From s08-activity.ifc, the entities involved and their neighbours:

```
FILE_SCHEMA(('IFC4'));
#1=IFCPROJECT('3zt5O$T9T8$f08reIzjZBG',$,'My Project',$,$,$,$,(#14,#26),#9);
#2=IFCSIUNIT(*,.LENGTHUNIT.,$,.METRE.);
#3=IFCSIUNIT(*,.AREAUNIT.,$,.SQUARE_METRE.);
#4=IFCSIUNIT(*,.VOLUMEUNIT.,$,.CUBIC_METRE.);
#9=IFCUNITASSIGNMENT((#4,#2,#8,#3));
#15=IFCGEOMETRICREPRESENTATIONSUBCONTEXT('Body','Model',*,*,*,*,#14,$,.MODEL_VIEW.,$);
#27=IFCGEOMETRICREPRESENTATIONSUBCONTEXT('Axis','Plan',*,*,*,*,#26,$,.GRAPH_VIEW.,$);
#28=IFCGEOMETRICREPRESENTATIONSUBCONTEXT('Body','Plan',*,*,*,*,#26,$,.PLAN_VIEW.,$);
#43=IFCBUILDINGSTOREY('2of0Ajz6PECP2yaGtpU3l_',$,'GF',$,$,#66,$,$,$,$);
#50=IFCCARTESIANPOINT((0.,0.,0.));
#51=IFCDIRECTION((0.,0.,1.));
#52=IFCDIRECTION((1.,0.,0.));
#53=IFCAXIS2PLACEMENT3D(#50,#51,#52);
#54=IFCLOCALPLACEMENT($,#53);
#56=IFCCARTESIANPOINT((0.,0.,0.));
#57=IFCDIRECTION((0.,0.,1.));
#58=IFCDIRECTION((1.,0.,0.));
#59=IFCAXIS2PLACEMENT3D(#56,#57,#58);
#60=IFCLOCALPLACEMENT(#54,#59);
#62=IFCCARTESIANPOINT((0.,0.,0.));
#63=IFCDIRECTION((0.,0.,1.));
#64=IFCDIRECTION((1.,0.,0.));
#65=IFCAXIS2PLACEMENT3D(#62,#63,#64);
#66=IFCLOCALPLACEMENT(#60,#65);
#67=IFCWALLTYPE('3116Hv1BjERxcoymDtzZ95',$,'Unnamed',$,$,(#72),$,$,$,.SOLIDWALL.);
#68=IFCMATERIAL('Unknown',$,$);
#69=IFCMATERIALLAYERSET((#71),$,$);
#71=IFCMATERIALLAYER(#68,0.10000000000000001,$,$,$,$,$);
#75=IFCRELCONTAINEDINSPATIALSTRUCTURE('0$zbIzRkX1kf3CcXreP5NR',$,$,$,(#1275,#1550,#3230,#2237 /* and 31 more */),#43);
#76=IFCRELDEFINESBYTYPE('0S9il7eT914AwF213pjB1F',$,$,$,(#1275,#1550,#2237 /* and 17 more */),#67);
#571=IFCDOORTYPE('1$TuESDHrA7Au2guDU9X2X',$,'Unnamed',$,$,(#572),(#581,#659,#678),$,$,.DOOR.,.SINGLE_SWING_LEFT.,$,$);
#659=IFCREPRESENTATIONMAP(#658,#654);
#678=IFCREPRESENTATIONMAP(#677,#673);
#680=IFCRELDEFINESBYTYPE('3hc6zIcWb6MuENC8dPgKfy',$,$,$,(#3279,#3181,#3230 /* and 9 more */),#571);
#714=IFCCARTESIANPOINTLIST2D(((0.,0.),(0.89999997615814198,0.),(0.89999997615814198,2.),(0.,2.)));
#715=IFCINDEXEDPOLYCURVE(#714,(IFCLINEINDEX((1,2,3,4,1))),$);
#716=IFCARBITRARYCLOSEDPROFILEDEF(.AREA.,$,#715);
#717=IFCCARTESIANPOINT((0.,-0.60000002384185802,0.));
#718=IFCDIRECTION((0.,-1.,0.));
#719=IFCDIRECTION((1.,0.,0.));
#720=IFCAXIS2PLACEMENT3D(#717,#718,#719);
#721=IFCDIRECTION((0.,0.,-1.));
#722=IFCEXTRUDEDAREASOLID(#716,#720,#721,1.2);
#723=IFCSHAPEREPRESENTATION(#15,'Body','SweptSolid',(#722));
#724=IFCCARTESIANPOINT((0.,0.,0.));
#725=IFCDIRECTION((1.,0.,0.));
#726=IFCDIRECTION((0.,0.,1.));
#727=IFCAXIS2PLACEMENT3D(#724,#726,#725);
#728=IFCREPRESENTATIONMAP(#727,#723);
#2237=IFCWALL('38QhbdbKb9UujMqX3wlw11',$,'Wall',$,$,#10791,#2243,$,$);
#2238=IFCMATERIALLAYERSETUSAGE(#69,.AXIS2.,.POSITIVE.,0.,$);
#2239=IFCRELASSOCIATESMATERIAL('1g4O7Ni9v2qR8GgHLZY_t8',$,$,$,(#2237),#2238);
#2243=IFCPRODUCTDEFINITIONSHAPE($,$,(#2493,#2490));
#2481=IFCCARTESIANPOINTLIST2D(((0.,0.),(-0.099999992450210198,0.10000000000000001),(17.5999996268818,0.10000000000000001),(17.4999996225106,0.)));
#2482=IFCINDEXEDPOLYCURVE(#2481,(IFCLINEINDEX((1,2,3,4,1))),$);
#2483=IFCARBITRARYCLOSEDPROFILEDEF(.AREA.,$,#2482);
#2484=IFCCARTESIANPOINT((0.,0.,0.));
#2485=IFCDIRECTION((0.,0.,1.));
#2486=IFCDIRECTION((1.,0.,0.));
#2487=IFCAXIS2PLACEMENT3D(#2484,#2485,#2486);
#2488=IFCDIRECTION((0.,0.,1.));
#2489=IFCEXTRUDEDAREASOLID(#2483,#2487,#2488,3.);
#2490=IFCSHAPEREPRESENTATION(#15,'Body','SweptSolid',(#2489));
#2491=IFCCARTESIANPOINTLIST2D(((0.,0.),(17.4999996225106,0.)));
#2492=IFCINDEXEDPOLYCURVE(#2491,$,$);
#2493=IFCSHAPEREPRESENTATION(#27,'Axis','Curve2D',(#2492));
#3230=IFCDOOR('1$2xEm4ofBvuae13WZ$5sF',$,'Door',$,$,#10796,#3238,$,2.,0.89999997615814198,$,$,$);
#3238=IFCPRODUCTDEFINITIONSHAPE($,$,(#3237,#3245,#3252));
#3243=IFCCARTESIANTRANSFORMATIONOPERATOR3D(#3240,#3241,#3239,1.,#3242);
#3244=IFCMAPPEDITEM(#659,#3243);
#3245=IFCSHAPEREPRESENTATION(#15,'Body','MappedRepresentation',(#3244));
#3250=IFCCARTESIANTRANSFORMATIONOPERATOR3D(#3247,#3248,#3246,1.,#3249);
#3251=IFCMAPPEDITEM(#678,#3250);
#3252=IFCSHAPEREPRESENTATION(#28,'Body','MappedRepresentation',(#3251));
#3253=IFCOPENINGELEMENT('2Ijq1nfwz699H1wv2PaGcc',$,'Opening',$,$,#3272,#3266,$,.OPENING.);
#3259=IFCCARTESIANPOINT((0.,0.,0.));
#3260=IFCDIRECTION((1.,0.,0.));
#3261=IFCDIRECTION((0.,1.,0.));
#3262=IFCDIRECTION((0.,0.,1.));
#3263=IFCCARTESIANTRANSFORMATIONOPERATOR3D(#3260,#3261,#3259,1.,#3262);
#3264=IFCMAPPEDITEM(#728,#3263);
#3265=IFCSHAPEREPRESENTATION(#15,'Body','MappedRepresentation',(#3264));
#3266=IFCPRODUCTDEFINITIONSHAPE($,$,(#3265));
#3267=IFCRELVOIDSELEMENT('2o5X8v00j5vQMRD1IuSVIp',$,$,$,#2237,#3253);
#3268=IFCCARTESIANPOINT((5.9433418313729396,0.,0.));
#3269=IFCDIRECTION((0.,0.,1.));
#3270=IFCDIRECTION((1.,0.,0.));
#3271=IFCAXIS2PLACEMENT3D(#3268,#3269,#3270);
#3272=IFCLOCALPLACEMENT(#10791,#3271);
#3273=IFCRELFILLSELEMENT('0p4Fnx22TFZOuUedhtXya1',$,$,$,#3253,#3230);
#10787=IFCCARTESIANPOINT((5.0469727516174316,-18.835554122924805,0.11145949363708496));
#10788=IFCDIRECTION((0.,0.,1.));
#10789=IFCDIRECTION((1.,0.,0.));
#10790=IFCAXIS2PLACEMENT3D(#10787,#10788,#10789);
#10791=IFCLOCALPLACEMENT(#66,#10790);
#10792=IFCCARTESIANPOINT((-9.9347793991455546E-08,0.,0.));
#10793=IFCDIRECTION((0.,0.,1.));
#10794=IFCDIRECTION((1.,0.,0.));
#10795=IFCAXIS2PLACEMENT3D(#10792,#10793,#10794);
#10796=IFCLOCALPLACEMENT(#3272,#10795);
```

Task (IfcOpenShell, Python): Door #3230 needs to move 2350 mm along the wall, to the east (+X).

```python
import ifcopenshell
import ifcopenshell.api.geometry
import ifcopenshell.util.placement
import ifcopenshell.util.unit

model = ifcopenshell.open("s08-activity.ifc")
unit_scale = ifcopenshell.util.unit.calculate_unit_scale(model)

door = model.by_id(3230)
opening = door.FillsVoids[0].RelatingOpeningElement
wall = opening.VoidsElements[0].RelatingBuildingElement

wall_matrix = ifcopenshell.util.placement.get_local_placement(wall.ObjectPlacement)
shift = wall_matrix[:3, 0] * 2.35 / unit_scale
before = ifcopenshell.util.placement.get_local_placement(door.ObjectPlacement)[:3, 3].copy()

# The door is placed relative to its opening, so it follows when the opening moves.
matrix = ifcopenshell.util.placement.get_local_placement(opening.ObjectPlacement)
matrix[:3, 3] += shift
ifcopenshell.api.geometry.edit_object_placement(
    model, product=opening, matrix=matrix, is_si=False, should_transform_children=True
)

after = ifcopenshell.util.placement.get_local_placement(door.ObjectPlacement)[:3, 3]
print("door moved by", (after - before).round(3) + 0.0)

model.write("s08-activity-out.ifc")
```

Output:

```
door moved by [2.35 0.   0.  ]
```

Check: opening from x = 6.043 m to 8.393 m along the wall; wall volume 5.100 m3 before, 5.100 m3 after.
